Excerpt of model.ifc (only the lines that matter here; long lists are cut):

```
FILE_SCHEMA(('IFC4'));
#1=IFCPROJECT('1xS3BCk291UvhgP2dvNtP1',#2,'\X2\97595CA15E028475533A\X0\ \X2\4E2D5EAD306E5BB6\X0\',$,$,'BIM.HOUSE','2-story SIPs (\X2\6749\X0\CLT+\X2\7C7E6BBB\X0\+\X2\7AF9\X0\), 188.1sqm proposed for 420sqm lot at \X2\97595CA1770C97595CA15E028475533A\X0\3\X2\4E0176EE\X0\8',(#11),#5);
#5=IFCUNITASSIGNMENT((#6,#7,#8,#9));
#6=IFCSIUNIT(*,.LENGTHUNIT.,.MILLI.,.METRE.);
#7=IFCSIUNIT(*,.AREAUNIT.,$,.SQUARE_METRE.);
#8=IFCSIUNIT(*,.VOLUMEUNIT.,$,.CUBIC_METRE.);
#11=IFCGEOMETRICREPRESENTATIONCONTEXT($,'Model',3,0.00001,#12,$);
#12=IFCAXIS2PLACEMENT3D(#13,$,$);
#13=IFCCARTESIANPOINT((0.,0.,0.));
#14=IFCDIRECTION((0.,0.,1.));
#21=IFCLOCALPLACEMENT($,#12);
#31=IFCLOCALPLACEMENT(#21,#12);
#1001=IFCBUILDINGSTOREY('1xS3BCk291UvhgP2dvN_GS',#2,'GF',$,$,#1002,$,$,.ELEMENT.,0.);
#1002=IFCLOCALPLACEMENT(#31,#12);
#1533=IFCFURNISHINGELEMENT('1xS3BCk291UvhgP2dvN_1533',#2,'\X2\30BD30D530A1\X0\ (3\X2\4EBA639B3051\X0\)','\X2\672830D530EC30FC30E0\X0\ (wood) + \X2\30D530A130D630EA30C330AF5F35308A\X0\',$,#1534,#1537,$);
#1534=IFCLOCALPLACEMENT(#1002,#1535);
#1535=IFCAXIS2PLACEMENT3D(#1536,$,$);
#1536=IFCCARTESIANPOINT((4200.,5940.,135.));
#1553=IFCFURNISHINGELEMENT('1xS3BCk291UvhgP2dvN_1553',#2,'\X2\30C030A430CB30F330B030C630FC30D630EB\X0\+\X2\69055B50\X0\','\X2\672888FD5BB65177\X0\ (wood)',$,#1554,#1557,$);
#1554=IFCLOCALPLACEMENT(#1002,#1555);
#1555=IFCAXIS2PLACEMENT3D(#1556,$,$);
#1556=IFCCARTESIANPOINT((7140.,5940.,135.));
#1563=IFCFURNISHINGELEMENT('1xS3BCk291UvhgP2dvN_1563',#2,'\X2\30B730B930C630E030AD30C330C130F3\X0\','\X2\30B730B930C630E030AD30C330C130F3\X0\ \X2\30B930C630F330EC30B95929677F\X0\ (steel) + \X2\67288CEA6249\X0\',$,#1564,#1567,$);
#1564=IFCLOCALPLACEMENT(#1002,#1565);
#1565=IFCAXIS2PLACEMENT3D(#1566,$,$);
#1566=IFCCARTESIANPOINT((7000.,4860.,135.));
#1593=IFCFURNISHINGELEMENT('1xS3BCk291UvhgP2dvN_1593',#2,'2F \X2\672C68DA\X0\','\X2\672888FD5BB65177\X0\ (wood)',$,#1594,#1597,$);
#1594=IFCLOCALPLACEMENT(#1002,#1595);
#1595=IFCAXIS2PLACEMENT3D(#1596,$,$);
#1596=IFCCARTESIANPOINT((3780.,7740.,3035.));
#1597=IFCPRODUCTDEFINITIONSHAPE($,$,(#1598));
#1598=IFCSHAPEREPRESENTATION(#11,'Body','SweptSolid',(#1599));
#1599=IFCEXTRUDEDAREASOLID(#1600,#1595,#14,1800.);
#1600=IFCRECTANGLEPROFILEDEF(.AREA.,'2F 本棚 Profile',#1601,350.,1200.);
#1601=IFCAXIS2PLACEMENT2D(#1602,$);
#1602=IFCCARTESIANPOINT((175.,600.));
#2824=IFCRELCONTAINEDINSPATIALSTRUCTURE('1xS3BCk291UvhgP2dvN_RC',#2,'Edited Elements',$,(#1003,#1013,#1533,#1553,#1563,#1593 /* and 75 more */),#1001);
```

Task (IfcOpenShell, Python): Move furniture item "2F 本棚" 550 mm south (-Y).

```python
import ifcopenshell
import ifcopenshell.api.geometry
import ifcopenshell.util.placement
import ifcopenshell.util.unit

model = ifcopenshell.open("model.ifc")
unit_scale = ifcopenshell.util.unit.calculate_unit_scale(model)

item = model.by_id(1593)
matrix = ifcopenshell.util.placement.get_local_placement(item.ObjectPlacement)
matrix[1, 3] -= 0.55 / unit_scale
ifcopenshell.api.geometry.edit_object_placement(model, product=item, matrix=matrix, is_si=False)

print(ifcopenshell.util.placement.get_local_placement(item.ObjectPlacement).round(3) + 0.0)

model.write("model_edited.ifc")
```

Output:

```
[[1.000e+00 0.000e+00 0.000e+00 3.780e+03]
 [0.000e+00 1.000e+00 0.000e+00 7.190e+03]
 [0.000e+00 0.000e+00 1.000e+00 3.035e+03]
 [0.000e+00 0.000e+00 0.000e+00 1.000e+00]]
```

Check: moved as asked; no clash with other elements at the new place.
